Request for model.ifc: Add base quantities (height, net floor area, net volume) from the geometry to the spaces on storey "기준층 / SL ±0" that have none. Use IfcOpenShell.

First a look at what the model holds.

```python
import ifcopenshell
import ifcopenshell.util.element
import ifcopenshell.util.unit

model = ifcopenshell.open("model.ifc")
print(model.schema)
for unit_type in ("LENGTHUNIT", "AREAUNIT", "VOLUMEUNIT"):
    print(unit_type, ifcopenshell.util.unit.calculate_unit_scale(model, unit_type))
storey = next(s for s in model.by_type("IfcBuildingStorey") if s.Name == "기준층 / SL ±0")
spaces = [e for e in ifcopenshell.util.element.get_decomposition(storey) if e.is_a("IfcSpace")]
for e in sorted(spaces, key=lambda e: e.id()):
    print(e.id(), e.is_a(), e.Name, list(ifcopenshell.util.element.get_psets(e, qtos_only=True)), sep=" | ")
```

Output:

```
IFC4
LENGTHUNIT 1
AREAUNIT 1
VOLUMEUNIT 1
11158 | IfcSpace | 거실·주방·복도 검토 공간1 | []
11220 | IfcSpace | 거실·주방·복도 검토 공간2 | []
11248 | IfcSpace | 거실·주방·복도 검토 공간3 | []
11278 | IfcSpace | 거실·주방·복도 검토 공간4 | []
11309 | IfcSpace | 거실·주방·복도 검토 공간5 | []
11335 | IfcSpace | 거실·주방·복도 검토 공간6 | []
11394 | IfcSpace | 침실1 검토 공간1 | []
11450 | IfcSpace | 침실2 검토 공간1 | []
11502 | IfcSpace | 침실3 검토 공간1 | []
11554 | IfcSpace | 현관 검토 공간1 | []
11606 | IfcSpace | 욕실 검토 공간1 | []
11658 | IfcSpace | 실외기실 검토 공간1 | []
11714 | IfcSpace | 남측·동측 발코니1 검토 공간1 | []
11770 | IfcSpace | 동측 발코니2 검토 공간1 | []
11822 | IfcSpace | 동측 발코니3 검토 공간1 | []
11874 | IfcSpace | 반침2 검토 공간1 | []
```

```python
import ifcopenshell
import ifcopenshell.api.pset
import ifcopenshell.geom
import ifcopenshell.util.element
import ifcopenshell.util.shape
import ifcopenshell.util.unit

model = ifcopenshell.open("model.ifc")
unit_scale = ifcopenshell.util.unit.calculate_unit_scale(model)
area_scale = ifcopenshell.util.unit.calculate_unit_scale(model, "AREAUNIT")
volume_scale = ifcopenshell.util.unit.calculate_unit_scale(model, "VOLUMEUNIT")
settings = ifcopenshell.geom.settings()

storey = next(s for s in model.by_type("IfcBuildingStorey") if s.Name == "기준층 / SL ±0")
spaces = [e for e in ifcopenshell.util.element.get_decomposition(storey) if e.is_a("IfcSpace")]

for e in sorted(spaces, key=lambda e: e.id()):
    if ifcopenshell.util.element.get_psets(e, qtos_only=True, should_inherit=False):
        continue
    # Geometry comes back in metres, in the element's own axes.
    shape = ifcopenshell.geom.create_shape(settings, e)
    values = {
        "Height": ifcopenshell.util.shape.get_z(shape.geometry) / unit_scale,
        "NetFloorArea": ifcopenshell.util.shape.get_footprint_area(shape.geometry) / area_scale,
        "NetVolume": ifcopenshell.util.shape.get_volume(shape.geometry) / volume_scale,
    }
    qto = ifcopenshell.api.pset.add_qto(model, product=e, name="Qto_SpaceBaseQuantities")
    ifcopenshell.api.pset.edit_qto(model, qto=qto, properties=values)
    print(e.id(), {k: round(v, 3) for k, v in values.items()})

model.write("model_updated.ifc")
```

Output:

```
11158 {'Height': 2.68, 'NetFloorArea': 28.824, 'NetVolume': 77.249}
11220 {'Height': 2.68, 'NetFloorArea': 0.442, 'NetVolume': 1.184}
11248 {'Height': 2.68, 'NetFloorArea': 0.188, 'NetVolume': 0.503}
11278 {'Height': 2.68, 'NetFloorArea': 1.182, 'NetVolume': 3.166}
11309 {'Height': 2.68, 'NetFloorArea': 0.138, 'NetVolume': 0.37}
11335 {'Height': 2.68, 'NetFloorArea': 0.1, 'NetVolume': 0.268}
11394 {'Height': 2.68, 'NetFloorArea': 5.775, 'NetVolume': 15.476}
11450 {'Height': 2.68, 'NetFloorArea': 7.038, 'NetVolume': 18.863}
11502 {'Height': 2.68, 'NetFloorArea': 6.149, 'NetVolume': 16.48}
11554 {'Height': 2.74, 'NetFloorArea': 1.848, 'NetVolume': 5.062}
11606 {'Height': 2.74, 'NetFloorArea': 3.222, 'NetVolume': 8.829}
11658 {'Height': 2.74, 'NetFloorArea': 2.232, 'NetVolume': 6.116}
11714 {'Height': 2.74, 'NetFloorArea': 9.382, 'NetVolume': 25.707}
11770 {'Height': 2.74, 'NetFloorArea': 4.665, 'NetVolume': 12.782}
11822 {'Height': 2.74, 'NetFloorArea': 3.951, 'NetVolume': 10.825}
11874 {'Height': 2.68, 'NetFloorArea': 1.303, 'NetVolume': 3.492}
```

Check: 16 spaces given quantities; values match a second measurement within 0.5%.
